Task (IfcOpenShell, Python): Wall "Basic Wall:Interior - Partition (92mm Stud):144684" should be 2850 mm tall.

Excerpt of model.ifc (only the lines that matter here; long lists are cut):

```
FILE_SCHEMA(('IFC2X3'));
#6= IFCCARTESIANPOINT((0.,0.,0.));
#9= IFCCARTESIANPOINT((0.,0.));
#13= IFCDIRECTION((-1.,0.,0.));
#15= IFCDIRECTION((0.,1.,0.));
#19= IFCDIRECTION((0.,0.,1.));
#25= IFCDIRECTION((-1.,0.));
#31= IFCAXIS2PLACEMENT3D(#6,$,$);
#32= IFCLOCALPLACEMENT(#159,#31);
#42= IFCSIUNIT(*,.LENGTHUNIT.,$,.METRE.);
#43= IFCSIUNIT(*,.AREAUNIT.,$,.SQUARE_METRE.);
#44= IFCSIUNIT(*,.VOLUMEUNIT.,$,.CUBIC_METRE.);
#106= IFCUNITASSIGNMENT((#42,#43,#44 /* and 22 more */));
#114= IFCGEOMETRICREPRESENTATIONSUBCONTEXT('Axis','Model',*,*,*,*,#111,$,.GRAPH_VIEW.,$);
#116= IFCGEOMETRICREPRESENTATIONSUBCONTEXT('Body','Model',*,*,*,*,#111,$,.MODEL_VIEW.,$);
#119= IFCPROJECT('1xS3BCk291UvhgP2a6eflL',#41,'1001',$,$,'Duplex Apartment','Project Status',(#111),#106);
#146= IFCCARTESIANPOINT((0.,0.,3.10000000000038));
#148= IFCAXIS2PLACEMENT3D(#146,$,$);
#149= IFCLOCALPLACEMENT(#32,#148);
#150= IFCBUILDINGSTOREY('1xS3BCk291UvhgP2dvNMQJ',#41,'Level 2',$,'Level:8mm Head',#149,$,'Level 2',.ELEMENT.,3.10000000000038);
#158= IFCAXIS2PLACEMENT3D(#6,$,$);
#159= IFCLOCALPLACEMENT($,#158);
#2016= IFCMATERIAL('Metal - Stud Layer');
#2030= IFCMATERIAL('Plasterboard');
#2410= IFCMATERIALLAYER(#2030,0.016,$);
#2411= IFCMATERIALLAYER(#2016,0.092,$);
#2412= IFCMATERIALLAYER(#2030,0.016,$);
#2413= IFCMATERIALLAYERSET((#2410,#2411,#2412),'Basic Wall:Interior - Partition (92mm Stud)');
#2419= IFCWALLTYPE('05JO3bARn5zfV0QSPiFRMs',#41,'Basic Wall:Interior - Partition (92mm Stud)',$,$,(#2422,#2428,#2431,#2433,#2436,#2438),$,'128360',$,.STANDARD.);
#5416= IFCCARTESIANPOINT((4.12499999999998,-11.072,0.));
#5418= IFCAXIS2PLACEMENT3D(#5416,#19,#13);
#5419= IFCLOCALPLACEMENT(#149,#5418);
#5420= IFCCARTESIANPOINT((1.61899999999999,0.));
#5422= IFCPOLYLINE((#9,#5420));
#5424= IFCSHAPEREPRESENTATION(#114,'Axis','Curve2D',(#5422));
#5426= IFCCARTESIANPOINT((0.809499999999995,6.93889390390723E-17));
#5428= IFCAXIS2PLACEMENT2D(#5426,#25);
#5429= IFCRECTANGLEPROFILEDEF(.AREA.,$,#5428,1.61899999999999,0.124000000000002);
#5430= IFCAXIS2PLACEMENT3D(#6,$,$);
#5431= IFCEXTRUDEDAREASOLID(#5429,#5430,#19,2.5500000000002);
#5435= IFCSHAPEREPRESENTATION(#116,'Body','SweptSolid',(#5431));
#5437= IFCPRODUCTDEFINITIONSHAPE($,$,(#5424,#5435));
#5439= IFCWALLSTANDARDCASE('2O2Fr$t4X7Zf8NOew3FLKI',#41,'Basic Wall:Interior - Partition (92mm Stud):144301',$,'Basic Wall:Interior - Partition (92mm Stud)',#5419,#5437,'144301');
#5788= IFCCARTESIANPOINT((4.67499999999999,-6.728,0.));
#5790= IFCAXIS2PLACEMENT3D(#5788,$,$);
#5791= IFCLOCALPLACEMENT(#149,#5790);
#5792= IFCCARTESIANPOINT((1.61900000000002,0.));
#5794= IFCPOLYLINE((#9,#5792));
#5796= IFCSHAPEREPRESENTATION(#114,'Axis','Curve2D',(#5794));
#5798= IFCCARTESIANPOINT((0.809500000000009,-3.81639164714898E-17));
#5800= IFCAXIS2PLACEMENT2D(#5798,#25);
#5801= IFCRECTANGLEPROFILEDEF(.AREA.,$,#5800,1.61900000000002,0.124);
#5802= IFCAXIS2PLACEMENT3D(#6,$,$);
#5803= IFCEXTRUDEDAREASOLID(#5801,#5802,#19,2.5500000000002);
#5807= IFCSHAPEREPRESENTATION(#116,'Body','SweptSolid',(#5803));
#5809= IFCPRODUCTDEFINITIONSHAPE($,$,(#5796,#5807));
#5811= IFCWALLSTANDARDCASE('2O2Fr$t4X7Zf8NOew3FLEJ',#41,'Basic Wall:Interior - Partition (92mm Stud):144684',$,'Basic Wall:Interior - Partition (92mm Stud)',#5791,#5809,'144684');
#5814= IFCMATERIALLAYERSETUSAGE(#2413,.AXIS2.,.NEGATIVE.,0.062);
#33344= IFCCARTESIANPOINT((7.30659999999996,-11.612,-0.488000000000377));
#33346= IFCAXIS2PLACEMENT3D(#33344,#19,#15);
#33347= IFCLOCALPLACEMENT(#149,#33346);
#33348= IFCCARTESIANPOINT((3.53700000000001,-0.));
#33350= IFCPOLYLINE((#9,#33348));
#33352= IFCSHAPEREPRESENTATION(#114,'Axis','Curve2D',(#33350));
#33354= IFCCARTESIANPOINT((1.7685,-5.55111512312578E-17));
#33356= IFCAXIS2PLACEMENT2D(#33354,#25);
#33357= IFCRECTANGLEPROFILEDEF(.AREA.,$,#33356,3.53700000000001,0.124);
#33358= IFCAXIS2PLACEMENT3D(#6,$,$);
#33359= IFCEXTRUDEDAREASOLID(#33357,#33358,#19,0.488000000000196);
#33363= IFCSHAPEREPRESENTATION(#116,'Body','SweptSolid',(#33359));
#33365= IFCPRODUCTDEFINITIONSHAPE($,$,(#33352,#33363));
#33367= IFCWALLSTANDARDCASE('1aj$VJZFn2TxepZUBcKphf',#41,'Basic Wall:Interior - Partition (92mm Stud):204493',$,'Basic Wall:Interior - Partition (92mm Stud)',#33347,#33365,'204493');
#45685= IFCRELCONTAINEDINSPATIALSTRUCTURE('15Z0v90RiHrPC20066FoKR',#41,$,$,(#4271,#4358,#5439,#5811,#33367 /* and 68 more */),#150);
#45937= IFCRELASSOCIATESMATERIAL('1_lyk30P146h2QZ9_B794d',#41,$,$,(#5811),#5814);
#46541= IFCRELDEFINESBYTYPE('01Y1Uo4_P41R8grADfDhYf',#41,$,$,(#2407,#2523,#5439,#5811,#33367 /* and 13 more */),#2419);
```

```python
import ifcopenshell
import ifcopenshell.geom
import ifcopenshell.util.representation
import ifcopenshell.util.shape
import ifcopenshell.util.unit

model = ifcopenshell.open("model.ifc")
unit_scale = ifcopenshell.util.unit.calculate_unit_scale(model)
settings = ifcopenshell.geom.settings()


def volume(element):
    """Net volume in cubic metres, openings subtracted."""
    shape = ifcopenshell.geom.create_shape(settings, element)
    return ifcopenshell.util.shape.get_volume(shape.geometry)


wall = model.by_guid("2O2Fr$t4X7Zf8NOew3FLEJ")
before = volume(wall)

body = ifcopenshell.util.representation.get_representation(wall, "Model", "Body")
solid = body.Items[0]
old_height = solid.Depth
solid.Depth = 2.85 / unit_scale
after = volume(wall)

print(f"height {old_height:g} -> {solid.Depth:g}, volume {before:.3f} -> {after:.3f} m3")

model.write("model_v2.ifc")
```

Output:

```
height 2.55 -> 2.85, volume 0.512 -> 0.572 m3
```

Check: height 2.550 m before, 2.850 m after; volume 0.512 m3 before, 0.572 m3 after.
